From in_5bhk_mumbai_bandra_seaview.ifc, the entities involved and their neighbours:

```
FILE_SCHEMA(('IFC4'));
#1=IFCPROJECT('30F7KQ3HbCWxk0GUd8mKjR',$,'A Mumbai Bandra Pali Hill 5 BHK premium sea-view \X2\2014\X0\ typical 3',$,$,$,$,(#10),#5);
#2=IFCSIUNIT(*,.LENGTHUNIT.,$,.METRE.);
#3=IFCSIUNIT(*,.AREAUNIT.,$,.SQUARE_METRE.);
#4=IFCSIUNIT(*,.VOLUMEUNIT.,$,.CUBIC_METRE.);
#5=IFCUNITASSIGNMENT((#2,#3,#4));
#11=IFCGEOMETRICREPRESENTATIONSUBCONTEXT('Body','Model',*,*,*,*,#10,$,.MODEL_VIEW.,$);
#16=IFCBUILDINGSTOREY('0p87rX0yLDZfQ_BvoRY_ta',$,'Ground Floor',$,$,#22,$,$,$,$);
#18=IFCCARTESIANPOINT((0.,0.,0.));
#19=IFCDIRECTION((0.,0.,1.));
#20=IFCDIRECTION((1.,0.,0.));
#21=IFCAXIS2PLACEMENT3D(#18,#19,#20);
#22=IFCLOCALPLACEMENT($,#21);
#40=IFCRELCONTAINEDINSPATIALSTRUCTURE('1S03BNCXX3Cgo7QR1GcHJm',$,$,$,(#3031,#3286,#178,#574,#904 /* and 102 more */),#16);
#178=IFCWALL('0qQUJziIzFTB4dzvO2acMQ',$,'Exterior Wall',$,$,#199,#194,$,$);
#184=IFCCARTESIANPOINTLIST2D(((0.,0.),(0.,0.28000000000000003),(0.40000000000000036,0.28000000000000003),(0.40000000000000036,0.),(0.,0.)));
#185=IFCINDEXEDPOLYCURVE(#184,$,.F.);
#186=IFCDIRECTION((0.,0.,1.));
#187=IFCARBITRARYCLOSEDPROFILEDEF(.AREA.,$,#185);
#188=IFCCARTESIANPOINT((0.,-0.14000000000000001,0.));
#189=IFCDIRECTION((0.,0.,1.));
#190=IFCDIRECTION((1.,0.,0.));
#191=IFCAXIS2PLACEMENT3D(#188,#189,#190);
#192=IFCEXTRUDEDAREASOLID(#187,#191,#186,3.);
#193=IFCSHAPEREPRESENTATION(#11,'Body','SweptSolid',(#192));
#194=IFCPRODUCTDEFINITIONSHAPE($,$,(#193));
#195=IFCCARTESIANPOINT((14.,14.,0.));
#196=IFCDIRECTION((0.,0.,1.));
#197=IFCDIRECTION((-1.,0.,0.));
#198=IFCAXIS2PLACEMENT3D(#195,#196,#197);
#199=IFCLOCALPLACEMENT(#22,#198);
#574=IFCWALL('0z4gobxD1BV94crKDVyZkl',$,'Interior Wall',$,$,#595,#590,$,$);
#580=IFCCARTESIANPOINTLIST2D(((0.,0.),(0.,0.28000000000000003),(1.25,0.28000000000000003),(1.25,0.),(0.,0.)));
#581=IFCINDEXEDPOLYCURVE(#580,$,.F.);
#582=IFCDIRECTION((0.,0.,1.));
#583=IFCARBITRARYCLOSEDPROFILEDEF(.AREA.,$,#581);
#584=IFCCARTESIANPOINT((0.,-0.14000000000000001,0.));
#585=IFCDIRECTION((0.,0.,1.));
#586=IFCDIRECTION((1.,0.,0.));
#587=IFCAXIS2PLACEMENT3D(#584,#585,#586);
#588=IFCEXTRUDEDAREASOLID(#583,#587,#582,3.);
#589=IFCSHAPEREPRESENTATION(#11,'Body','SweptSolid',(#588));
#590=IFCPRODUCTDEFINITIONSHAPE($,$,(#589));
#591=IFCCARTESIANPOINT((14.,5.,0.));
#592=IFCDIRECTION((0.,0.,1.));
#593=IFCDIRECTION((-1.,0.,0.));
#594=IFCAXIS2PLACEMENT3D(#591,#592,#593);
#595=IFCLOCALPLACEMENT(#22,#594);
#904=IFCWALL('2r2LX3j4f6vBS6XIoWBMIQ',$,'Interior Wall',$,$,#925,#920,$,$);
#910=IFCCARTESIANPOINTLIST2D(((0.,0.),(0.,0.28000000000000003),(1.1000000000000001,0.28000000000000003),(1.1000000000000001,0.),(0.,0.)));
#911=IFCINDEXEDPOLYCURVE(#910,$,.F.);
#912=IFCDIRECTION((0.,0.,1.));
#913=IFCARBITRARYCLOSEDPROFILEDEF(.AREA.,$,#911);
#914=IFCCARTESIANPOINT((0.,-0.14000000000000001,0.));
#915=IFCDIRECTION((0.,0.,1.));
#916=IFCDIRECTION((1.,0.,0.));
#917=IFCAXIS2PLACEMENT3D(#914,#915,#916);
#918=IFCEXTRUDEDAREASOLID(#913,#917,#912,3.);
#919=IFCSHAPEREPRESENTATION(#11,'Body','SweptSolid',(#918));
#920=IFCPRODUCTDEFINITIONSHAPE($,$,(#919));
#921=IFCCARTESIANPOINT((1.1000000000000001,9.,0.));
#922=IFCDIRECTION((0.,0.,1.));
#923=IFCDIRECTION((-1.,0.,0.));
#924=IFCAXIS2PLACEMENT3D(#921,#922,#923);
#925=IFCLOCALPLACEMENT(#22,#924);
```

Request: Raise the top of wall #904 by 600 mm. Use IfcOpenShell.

```python
import ifcopenshell
import ifcopenshell.geom
import ifcopenshell.util.representation
import ifcopenshell.util.shape
import ifcopenshell.util.unit

model = ifcopenshell.open("in_5bhk_mumbai_bandra_seaview.ifc")
unit_scale = ifcopenshell.util.unit.calculate_unit_scale(model)
settings = ifcopenshell.geom.settings()


def volume(element):
    """Net volume in cubic metres, openings subtracted."""
    shape = ifcopenshell.geom.create_shape(settings, element)
    return ifcopenshell.util.shape.get_volume(shape.geometry)


wall = model.by_guid("2r2LX3j4f6vBS6XIoWBMIQ")
before = volume(wall)

body = ifcopenshell.util.representation.get_representation(wall, "Model", "Body")
solid = body.Items[0]
old_height = solid.Depth
solid.Depth += 0.6 / unit_scale
after = volume(wall)

print(f"height {old_height:g} -> {solid.Depth:g}, volume {before:.3f} -> {after:.3f} m3")

model.write("in_5bhk_mumbai_bandra_seaview-out.ifc")
```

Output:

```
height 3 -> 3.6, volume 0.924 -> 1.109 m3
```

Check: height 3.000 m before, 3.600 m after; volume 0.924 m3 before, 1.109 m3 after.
